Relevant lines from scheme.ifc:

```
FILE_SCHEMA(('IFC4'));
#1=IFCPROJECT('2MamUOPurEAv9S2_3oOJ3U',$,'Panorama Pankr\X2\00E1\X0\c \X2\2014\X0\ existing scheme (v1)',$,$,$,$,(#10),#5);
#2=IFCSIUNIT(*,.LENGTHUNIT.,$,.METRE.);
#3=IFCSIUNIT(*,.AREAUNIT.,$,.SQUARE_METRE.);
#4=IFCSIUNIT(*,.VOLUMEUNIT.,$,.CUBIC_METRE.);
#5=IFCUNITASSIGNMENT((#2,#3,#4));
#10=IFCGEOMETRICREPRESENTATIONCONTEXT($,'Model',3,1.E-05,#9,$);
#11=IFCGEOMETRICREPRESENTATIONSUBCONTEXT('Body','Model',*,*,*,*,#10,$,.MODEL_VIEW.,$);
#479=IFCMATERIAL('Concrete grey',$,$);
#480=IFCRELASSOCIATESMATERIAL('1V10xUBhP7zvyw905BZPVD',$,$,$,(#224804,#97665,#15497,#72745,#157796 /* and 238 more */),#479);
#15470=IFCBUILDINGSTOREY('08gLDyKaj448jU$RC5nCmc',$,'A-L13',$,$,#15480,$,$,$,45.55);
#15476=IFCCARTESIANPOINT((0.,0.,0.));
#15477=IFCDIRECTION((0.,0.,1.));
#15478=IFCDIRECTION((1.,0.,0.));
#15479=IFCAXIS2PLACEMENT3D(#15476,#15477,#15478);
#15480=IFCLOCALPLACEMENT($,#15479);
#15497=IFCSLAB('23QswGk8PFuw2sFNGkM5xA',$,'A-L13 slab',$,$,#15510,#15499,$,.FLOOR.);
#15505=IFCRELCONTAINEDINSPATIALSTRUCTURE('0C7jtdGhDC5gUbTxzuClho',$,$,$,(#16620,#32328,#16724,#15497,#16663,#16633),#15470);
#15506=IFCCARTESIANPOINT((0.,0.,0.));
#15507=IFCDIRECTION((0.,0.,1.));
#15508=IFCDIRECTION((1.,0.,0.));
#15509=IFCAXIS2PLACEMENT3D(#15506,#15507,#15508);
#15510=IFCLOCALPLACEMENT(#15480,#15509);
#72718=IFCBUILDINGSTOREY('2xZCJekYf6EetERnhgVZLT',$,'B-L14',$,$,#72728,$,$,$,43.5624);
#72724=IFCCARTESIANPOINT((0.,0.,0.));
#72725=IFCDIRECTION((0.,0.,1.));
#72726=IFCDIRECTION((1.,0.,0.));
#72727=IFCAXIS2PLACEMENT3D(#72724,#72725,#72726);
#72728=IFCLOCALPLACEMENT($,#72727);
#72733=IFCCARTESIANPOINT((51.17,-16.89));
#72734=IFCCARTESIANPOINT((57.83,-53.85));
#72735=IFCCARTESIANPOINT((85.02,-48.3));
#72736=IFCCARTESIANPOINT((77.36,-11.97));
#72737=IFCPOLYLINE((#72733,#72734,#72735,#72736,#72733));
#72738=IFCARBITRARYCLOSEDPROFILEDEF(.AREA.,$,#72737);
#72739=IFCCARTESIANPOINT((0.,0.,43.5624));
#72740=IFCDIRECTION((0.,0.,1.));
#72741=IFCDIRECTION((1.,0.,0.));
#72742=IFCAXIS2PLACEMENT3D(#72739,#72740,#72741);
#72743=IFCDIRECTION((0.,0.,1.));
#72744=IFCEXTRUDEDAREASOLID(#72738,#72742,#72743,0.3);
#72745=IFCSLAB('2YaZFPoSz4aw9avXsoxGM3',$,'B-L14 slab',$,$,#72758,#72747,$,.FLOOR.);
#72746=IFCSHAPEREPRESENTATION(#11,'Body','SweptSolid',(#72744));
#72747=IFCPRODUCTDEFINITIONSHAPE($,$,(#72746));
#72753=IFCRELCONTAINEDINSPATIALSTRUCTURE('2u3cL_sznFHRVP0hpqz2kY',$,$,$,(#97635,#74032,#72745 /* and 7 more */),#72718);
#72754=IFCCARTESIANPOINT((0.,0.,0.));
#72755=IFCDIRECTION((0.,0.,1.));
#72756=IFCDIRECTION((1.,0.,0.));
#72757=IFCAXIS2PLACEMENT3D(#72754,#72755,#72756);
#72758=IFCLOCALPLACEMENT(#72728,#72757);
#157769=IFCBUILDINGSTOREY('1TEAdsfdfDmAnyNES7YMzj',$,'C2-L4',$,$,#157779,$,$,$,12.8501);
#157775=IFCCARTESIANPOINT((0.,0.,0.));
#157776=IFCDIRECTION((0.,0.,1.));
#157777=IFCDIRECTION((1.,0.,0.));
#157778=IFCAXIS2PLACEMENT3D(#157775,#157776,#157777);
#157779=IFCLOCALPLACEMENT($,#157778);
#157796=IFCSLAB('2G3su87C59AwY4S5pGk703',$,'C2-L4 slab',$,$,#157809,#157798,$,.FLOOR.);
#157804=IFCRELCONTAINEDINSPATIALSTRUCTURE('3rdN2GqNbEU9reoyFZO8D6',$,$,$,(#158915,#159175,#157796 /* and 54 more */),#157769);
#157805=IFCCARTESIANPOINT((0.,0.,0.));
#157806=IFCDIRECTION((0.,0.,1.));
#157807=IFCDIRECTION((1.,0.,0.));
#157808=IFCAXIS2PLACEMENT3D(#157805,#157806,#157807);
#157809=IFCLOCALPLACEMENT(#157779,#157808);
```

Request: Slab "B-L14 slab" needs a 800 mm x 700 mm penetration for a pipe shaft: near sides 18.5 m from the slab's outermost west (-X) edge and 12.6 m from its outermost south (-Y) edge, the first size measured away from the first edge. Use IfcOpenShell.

```python
import numpy as np
import ifcopenshell
import ifcopenshell.api.feature
import ifcopenshell.api.geometry
import ifcopenshell.api.root
import ifcopenshell.geom
import ifcopenshell.util.placement
import ifcopenshell.util.representation
import ifcopenshell.util.shape
import ifcopenshell.util.unit

model = ifcopenshell.open("scheme.ifc")
unit_scale = ifcopenshell.util.unit.calculate_unit_scale(model)
settings = ifcopenshell.geom.settings()


def volume(element):
    """Net volume in cubic metres, openings subtracted."""
    shape = ifcopenshell.geom.create_shape(settings, element)
    return ifcopenshell.util.shape.get_volume(shape.geometry)


slab = model.by_id(72745)
before = volume(slab)

# Extent in the slab's own axes, in metres. The edges named are its -X and -Y sides.
slab_shape = ifcopenshell.geom.create_shape(settings, slab)
vertices = ifcopenshell.util.shape.get_vertices(slab_shape.geometry)
x_min, y_min, bottom = vertices.min(axis=0)
top = vertices[:, 2].max()

opening = ifcopenshell.api.root.create_entity(model, ifc_class="IfcOpeningElement", name="Pipe shaft opening", predefined_type="OPENING")
context = ifcopenshell.util.representation.get_context(model, "Model", "Body", "MODEL_VIEW")
width, depth = 0.8, 0.7
outline = [(0.0, 0.0), (width, 0.0), (width, depth), (0.0, depth), (0.0, 0.0)]
# Overshoot both faces by 50 mm so the cut is clean.
shape = ifcopenshell.api.geometry.add_slab_representation(
    model, context=context, depth=top - bottom + 0.1, polyline=outline
)
ifcopenshell.api.geometry.assign_representation(model, product=opening, representation=shape)

matrix = ifcopenshell.util.placement.get_local_placement(slab.ObjectPlacement)
matrix[:, 3] = matrix @ np.append(np.array([x_min + 18.5, y_min + 12.6, bottom - 0.05]) / unit_scale, 1.0)
ifcopenshell.api.geometry.edit_object_placement(model, product=opening, matrix=matrix, is_si=False)
ifcopenshell.api.feature.add_feature(model, feature=opening, element=slab)

after = volume(slab)

print(f"slab volume {before:.3f} -> {after:.3f} m3")

model.write("scheme_edited.ifc")
```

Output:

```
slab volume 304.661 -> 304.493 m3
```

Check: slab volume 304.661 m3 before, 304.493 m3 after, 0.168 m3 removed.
